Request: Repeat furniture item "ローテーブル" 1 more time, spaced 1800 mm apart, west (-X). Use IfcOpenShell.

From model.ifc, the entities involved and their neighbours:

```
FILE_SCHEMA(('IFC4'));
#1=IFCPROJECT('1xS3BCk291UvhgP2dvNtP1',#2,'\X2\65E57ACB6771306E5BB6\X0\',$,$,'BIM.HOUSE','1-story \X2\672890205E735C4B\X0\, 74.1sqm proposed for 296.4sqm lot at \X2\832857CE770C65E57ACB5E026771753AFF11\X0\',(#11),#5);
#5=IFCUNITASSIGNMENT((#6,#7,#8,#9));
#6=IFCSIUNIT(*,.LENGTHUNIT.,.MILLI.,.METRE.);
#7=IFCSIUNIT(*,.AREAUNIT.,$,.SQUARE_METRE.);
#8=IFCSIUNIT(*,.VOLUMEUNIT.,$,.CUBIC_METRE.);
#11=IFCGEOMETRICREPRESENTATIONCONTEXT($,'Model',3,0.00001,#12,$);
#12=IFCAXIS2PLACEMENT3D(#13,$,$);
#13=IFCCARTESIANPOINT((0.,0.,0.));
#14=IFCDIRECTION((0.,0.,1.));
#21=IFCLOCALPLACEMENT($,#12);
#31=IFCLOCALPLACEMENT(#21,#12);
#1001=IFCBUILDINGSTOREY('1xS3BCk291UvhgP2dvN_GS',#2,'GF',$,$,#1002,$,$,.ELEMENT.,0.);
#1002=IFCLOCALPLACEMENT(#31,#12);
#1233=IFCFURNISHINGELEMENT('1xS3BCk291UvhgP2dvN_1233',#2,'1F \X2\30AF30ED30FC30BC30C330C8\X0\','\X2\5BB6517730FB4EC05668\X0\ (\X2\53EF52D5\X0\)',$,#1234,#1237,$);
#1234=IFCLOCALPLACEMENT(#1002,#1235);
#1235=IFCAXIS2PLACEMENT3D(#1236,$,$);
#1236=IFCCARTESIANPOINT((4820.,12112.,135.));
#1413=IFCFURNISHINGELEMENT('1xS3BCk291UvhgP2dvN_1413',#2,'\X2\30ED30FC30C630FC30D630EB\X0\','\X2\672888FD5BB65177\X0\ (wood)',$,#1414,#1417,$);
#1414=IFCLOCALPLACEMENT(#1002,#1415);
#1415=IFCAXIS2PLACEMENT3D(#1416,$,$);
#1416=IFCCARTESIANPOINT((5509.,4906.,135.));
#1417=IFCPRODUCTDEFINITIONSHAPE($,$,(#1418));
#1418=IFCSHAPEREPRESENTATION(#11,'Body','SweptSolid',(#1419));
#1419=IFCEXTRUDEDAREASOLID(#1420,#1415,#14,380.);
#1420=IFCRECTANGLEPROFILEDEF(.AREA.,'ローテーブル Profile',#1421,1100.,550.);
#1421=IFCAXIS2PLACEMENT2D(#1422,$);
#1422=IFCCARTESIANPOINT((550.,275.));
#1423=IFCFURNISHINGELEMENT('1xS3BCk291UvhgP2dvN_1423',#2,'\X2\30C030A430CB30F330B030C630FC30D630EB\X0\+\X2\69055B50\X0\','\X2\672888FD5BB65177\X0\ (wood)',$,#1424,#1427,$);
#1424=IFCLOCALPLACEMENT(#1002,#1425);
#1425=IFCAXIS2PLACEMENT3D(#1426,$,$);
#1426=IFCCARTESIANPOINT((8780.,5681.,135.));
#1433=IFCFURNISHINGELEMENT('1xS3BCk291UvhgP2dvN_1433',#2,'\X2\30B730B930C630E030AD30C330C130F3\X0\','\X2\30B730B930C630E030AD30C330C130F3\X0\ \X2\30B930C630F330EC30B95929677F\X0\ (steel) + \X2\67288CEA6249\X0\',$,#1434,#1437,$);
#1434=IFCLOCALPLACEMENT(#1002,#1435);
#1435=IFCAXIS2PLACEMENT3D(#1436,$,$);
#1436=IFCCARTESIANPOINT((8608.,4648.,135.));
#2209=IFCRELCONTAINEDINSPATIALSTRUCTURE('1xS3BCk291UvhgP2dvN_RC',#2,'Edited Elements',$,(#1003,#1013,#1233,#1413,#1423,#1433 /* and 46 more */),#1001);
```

```python
import numpy as np
import ifcopenshell
import ifcopenshell.api.geometry
import ifcopenshell.api.root
import ifcopenshell.util.element
import ifcopenshell.util.placement
import ifcopenshell.util.unit

model = ifcopenshell.open("model.ifc")
unit_scale = ifcopenshell.util.unit.calculate_unit_scale(model)


def reuse_history(source, copy):
    """copy_class also copies each property set's owner history, people and application; keep the originals."""
    for rel in copy.IsDefinedBy:
        if rel.is_a("IfcRelDefinesByProperties") and (history := rel.RelatingPropertyDefinition.OwnerHistory):
            rel.RelatingPropertyDefinition.OwnerHistory = source.OwnerHistory
            ifcopenshell.util.element.remove_deep2(model, history)


source = model.by_guid("1xS3BCk291UvhgP2dvN_1413")
base = ifcopenshell.util.placement.get_local_placement(source.ObjectPlacement)
step = np.array([-1.0, 0.0, 0.0]) * 1.8 / unit_scale

for i in range(1, 2):
    copy = ifcopenshell.api.root.copy_class(model, product=source)
    copy.Representation = ifcopenshell.util.element.copy_deep(
        model, source.Representation, exclude=["IfcGeometricRepresentationContext", "IfcRepresentationMap"]
    )
    reuse_history(source, copy)
    matrix = base.copy()
    matrix[:3, 3] += i * step
    print("added at", matrix[:3, 3].round(3) + 0.0)
    ifcopenshell.api.geometry.edit_object_placement(model, product=copy, matrix=matrix, is_si=False)

model.write("model_rev.ifc")
```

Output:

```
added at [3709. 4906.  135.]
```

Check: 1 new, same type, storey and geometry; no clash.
